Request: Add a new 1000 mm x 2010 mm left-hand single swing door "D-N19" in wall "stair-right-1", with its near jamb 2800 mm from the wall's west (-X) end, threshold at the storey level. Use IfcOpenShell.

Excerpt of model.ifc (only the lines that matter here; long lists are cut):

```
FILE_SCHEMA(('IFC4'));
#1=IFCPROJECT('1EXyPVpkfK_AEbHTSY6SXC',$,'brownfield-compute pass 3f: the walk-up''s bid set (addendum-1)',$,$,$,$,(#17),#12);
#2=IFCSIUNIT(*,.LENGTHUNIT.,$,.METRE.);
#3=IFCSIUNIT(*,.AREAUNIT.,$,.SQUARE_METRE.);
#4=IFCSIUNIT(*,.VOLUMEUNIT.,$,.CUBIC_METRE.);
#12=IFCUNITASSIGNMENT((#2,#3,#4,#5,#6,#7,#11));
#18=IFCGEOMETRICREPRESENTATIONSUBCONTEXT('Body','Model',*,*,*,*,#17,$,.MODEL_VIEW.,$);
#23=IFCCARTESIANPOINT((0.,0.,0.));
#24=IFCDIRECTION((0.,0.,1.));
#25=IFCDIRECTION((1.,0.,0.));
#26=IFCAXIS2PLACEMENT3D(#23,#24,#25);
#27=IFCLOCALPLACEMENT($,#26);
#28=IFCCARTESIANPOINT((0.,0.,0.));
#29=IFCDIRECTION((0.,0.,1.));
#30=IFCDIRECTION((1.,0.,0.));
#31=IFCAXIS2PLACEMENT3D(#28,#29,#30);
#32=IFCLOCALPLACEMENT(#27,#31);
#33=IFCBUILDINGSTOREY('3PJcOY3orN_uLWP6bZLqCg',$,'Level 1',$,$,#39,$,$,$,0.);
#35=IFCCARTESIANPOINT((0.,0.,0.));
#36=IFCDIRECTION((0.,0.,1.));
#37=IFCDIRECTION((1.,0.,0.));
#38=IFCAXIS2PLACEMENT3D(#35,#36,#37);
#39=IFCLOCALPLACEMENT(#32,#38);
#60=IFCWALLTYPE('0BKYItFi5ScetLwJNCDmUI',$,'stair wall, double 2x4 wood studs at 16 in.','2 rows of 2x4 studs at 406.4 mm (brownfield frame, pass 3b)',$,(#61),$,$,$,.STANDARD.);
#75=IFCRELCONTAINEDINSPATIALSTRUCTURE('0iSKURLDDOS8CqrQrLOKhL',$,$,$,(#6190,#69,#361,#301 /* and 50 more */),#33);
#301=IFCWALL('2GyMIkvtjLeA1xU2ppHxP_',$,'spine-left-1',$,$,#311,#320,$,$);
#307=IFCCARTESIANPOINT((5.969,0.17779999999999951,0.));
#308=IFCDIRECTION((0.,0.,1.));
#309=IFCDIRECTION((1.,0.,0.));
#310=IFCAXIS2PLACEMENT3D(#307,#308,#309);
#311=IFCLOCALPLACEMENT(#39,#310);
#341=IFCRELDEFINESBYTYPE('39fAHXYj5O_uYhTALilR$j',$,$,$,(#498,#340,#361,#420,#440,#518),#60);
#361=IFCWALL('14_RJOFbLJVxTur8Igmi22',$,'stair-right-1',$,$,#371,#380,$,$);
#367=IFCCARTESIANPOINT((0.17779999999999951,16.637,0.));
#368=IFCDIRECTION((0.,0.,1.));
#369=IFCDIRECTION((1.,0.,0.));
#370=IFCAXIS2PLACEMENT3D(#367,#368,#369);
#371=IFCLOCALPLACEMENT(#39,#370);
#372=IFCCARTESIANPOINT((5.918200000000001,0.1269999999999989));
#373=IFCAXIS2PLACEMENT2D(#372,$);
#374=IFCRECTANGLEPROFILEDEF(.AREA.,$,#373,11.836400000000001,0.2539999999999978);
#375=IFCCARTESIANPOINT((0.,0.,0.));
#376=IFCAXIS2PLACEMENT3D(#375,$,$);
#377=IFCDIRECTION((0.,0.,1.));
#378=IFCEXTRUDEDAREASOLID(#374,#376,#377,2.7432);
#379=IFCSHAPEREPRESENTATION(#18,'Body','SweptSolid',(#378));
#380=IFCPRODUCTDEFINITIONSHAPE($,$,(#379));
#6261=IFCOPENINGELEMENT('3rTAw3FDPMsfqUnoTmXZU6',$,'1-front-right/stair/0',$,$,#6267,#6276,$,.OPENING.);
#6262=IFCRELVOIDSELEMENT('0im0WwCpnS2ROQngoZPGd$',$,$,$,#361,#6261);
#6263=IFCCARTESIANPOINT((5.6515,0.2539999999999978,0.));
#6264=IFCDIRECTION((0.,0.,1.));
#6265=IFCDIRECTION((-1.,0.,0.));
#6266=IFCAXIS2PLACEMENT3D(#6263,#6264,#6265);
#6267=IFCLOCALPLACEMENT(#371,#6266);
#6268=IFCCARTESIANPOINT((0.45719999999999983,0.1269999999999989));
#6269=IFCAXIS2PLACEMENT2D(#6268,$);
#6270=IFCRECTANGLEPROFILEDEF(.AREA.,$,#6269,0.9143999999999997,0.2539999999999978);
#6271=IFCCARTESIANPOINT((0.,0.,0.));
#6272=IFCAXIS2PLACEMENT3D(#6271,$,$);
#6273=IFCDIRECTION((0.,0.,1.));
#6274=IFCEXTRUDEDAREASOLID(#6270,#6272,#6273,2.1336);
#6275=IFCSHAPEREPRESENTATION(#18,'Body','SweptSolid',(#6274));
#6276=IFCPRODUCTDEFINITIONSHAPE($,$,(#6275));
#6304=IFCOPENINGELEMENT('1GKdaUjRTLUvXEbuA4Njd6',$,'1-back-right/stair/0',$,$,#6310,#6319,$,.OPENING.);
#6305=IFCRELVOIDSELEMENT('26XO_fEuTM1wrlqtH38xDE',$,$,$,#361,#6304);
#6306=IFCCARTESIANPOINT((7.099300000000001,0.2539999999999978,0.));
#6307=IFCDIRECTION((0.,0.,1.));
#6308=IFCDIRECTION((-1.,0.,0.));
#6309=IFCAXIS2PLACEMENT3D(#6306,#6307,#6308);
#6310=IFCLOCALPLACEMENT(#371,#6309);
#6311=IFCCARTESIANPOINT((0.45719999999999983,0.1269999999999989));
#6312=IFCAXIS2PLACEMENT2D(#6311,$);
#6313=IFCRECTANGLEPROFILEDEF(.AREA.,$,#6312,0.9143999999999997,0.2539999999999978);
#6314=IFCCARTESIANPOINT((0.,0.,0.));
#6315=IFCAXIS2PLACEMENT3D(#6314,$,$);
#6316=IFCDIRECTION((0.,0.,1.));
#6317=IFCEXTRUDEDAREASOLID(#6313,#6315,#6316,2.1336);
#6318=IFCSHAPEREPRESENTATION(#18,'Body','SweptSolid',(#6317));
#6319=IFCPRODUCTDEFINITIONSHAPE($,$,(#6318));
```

```python
import numpy as np
import ifcopenshell
import ifcopenshell.api.feature
import ifcopenshell.api.geometry
import ifcopenshell.api.root
import ifcopenshell.api.spatial
import ifcopenshell.geom
import ifcopenshell.util.element
import ifcopenshell.util.placement
import ifcopenshell.util.representation
import ifcopenshell.util.shape
import ifcopenshell.util.unit

model = ifcopenshell.open("model.ifc")
unit_scale = ifcopenshell.util.unit.calculate_unit_scale(model)
settings = ifcopenshell.geom.settings()


def volume(element):
    """Net volume in cubic metres, openings subtracted."""
    shape = ifcopenshell.geom.create_shape(settings, element)
    return ifcopenshell.util.shape.get_volume(shape.geometry)


wall = model.by_guid("14_RJOFbLJVxTur8Igmi22")
storey = ifcopenshell.util.element.get_container(wall, ifc_class="IfcBuildingStorey")
context = ifcopenshell.util.representation.get_context(model, "Model", "Body", "MODEL_VIEW")
before = volume(wall)

width, height, from_end, sill = 1, 2.01, 2.8, 0.0  # metres

# The wall runs along its own X axis, and the end named is its -X end.
wall_shape = ifcopenshell.geom.create_shape(settings, wall)
x, y, z = ifcopenshell.util.shape.get_vertices(wall_shape.geometry).T
start = x.min() + from_end
face, thickness = float(y.min()), float(y.max() - y.min())
wall_matrix = ifcopenshell.util.placement.get_local_placement(wall.ObjectPlacement)
level = ifcopenshell.util.placement.get_local_placement(storey.ObjectPlacement)[2, 3]


def in_wall(x, y):
    """Placement at x, y metres in the wall's axes, at sill height."""
    matrix = wall_matrix.copy()
    matrix[:, 3] = wall_matrix @ np.array([x / unit_scale, y / unit_scale, 0.0, 1.0])
    matrix[2, 3] = level + sill / unit_scale
    return matrix


# Opening: a box that overshoots both wall faces by 50 mm.
opening = ifcopenshell.api.root.create_entity(model, ifc_class="IfcOpeningElement", predefined_type="OPENING")
box = ifcopenshell.api.geometry.add_wall_representation(
    model, context=context, length=width, height=height, thickness=thickness + 0.1
)
ifcopenshell.api.geometry.assign_representation(model, product=opening, representation=box)
ifcopenshell.api.geometry.edit_object_placement(model, product=opening, matrix=in_wall(start, face - 0.05), is_si=False)
ifcopenshell.api.feature.add_feature(model, feature=opening, element=wall)

door = ifcopenshell.api.root.create_entity(model, ifc_class="IfcDoor", name="D-N19", predefined_type="DOOR")
door.OverallWidth, door.OverallHeight = width / unit_scale, height / unit_scale
door.OperationType = "SINGLE_SWING_LEFT"
body = ifcopenshell.api.geometry.add_door_representation(
    model,
    context=context,
    overall_width=door.OverallWidth,
    overall_height=door.OverallHeight,
    operation_type="SINGLE_SWING_LEFT",
    lining_properties={"LiningDepth": thickness / unit_scale, "ThresholdDepth": thickness / unit_scale},
)
ifcopenshell.api.geometry.assign_representation(model, product=door, representation=body)
ifcopenshell.api.spatial.assign_container(model, products=[door], relating_structure=storey)
ifcopenshell.api.feature.add_filling(model, opening=opening, element=door)

# The lining spans the wall, so the door starts at the wall face.
ifcopenshell.api.geometry.edit_object_placement(model, product=door, matrix=in_wall(start, face), is_si=False)

after = volume(wall)

print(f"wall volume {before:.3f} -> {after:.3f} m3")

model.write("model_rev.ifc")
```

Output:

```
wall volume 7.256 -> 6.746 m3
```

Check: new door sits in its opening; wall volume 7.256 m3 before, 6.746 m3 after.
